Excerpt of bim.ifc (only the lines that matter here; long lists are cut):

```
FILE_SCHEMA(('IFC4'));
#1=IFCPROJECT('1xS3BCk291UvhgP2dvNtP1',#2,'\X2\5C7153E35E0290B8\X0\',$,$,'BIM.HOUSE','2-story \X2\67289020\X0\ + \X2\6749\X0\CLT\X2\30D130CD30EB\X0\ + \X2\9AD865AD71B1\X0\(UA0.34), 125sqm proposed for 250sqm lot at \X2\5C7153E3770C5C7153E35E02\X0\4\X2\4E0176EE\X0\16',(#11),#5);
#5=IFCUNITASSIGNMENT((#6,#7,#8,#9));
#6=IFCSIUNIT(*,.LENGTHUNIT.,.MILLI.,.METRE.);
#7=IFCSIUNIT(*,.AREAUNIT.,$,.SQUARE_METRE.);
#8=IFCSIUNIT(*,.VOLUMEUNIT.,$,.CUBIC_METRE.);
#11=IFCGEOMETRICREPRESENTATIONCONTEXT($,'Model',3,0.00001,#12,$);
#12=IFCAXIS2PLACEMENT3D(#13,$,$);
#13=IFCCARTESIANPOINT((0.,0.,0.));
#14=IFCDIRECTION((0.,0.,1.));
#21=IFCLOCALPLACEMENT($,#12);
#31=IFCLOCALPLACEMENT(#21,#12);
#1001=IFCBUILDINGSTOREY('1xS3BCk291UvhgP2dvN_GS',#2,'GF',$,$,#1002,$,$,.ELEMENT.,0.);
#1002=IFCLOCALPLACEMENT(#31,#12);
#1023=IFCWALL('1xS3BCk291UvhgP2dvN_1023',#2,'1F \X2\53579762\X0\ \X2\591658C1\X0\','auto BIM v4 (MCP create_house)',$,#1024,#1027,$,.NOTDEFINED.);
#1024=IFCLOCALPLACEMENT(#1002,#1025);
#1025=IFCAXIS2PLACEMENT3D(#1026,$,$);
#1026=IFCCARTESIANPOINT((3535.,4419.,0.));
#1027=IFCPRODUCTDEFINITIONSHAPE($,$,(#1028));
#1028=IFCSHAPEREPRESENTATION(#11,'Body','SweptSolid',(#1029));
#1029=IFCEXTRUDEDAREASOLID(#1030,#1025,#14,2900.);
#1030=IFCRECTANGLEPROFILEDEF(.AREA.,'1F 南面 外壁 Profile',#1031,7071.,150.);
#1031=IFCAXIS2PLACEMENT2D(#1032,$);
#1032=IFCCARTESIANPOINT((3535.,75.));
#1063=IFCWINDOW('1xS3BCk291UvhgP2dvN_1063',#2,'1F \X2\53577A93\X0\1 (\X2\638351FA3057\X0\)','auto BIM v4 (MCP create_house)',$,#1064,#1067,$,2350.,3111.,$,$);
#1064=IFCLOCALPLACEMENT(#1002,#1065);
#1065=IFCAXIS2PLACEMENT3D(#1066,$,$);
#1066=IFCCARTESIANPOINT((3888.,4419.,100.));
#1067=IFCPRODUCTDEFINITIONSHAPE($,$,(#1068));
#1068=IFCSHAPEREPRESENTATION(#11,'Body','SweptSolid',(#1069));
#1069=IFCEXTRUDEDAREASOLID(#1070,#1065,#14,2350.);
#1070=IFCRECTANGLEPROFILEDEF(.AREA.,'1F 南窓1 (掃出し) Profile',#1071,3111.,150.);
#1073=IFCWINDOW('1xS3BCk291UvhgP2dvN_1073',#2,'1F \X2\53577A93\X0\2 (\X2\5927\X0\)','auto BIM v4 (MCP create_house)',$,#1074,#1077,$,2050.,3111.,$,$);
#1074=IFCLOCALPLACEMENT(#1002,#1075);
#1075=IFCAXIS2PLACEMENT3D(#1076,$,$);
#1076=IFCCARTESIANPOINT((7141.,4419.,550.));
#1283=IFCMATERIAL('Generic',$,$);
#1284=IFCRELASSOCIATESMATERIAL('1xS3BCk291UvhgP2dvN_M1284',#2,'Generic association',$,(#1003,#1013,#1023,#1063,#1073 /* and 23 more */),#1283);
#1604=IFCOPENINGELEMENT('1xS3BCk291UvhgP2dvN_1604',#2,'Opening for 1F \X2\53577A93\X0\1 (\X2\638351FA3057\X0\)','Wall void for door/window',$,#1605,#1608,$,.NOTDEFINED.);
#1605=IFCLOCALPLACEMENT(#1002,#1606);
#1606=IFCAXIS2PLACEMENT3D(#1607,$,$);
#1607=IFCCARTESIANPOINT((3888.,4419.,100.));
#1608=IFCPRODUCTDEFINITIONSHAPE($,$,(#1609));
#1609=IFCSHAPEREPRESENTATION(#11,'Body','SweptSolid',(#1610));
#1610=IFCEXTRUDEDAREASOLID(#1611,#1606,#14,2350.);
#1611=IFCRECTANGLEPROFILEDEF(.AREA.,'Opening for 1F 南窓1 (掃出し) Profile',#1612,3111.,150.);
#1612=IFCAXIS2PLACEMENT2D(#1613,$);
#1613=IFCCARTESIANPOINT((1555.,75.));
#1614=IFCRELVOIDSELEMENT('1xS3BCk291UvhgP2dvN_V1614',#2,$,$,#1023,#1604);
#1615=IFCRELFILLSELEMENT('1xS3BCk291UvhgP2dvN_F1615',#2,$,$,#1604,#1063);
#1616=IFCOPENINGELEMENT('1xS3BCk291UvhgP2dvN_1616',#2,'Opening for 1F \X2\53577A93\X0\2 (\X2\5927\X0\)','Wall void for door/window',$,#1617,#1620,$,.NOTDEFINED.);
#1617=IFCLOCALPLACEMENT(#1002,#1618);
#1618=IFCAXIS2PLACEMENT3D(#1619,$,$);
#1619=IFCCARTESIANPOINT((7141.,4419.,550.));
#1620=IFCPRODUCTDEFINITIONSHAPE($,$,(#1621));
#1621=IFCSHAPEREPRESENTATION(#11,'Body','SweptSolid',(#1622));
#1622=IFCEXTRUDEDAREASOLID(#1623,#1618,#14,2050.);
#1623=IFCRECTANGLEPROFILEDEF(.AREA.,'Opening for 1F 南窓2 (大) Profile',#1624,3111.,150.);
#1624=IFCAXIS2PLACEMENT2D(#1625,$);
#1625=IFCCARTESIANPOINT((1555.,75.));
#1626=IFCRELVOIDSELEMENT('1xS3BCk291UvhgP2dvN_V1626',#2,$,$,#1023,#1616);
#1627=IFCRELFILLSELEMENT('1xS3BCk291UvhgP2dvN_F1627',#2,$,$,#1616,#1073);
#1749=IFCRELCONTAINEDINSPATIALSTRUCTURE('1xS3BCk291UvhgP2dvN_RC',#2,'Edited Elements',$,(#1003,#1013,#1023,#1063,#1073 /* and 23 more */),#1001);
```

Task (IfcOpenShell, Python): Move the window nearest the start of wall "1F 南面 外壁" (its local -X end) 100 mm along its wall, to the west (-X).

```python
import ifcopenshell
import ifcopenshell.api.geometry
import ifcopenshell.util.placement

model = ifcopenshell.open("bim.ifc")

window = model.by_guid("1xS3BCk291UvhgP2dvN_1063")
opening = window.FillsVoids[0].RelatingOpeningElement
wall = opening.VoidsElements[0].RelatingBuildingElement

wall_matrix = ifcopenshell.util.placement.get_local_placement(wall.ObjectPlacement)
shift = wall_matrix[:3, 0] * -100.0
before = ifcopenshell.util.placement.get_local_placement(window.ObjectPlacement)[:3, 3].copy()

# The window is not placed relative to its opening, so move both.
for product in (opening, window):
    matrix = ifcopenshell.util.placement.get_local_placement(product.ObjectPlacement)
    matrix[:3, 3] += shift
    ifcopenshell.api.geometry.edit_object_placement(model, product=product, matrix=matrix, is_si=False)

after = ifcopenshell.util.placement.get_local_placement(window.ObjectPlacement)[:3, 3]
print("window moved by", (after - before).round(3) + 0.0)

model.write("bim_updated.ifc")
```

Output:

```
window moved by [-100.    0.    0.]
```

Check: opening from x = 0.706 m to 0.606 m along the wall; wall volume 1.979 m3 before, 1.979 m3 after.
